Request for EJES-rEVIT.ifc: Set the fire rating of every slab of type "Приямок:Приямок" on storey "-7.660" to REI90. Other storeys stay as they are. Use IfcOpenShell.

First a look at what the model holds.

```python
import ifcopenshell
import ifcopenshell.util.element

model = ifcopenshell.open("EJES-rEVIT.ifc")
print(model.schema)
storey = next(s for s in model.by_type("IfcBuildingStorey") if s.Name == "-7.660")
slabs = [e for e in ifcopenshell.util.element.get_decomposition(storey) if e.is_a("IfcSlab")]
seen = {}
for e in slabs:
    element_type = ifcopenshell.util.element.get_type(e)
    key = (element_type.Name if element_type != e and element_type else None, ifcopenshell.util.element.get_pset(e, "Pset_SlabCommon", "FireRating"))
    seen[key] = seen.get(key, 0) + 1
for (name, value), count in sorted(seen.items(), key=str):
    print(count, "x", name, "|", value)
```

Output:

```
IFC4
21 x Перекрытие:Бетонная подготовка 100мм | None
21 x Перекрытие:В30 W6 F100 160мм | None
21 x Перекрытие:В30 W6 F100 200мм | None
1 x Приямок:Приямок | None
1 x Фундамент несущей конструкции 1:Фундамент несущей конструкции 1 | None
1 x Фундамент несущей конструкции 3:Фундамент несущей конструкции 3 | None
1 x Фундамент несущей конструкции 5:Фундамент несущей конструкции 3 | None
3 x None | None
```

```python
import ifcopenshell
import ifcopenshell.api.pset
import ifcopenshell.util.element

model = ifcopenshell.open("EJES-rEVIT.ifc")

storey = next(s for s in model.by_type("IfcBuildingStorey") if s.Name == "-7.660")
slabs = [e for e in ifcopenshell.util.element.get_decomposition(storey) if e.is_a("IfcSlab")]

count = 0
for e in slabs:
    element_type = ifcopenshell.util.element.get_type(e)
    if element_type in (None, e) or element_type.Name != "Приямок:Приямок":
        continue
    # add_pset returns the element's existing set when there is one.
    pset = ifcopenshell.api.pset.add_pset(model, product=e, name="Pset_SlabCommon")
    ifcopenshell.api.pset.edit_pset(model, pset=pset, properties={"FireRating": "REI90"})
    count += 1

print(count, "slabs updated")

model.write("EJES-rEVIT_rev.ifc")
```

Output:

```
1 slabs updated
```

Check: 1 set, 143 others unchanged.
